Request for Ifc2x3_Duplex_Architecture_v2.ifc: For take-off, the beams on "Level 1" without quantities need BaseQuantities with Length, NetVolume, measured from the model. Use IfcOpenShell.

First a look at what the model holds.

```python
import ifcopenshell
import ifcopenshell.util.element
import ifcopenshell.util.unit

model = ifcopenshell.open("Ifc2x3_Duplex_Architecture_v2.ifc")
print(model.schema)
for unit_type in ("LENGTHUNIT", "AREAUNIT", "VOLUMEUNIT"):
    print(unit_type, ifcopenshell.util.unit.calculate_unit_scale(model, unit_type))
storey = next(s for s in model.by_type("IfcBuildingStorey") if s.Name == "Level 1")
beams = [e for e in ifcopenshell.util.element.get_decomposition(storey) if e.is_a("IfcBeam")]
for e in sorted(beams, key=lambda e: e.id()):
    print(e.id(), e.is_a(), e.Name, list(ifcopenshell.util.element.get_psets(e, qtos_only=True)), sep=" | ")
```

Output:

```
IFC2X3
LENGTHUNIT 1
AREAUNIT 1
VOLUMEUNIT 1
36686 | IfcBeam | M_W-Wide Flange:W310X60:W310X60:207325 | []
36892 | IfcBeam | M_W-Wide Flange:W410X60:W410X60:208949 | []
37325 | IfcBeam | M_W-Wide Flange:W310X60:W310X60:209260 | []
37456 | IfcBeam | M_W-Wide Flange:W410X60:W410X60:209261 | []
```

```python
import ifcopenshell
import ifcopenshell.api.pset
import ifcopenshell.geom
import ifcopenshell.util.element
import ifcopenshell.util.shape
import ifcopenshell.util.unit

model = ifcopenshell.open("Ifc2x3_Duplex_Architecture_v2.ifc")
unit_scale = ifcopenshell.util.unit.calculate_unit_scale(model)
volume_scale = ifcopenshell.util.unit.calculate_unit_scale(model, "VOLUMEUNIT")
settings = ifcopenshell.geom.settings()

storey = next(s for s in model.by_type("IfcBuildingStorey") if s.Name == "Level 1")
beams = [e for e in ifcopenshell.util.element.get_decomposition(storey) if e.is_a("IfcBeam")]

for e in sorted(beams, key=lambda e: e.id()):
    if ifcopenshell.util.element.get_psets(e, qtos_only=True, should_inherit=False):
        continue
    # Geometry comes back in metres, in the element's own axes.
    shape = ifcopenshell.geom.create_shape(settings, e)
    values = {
        "Length": ifcopenshell.util.shape.get_max_xyz(shape.geometry) / unit_scale,
        "NetVolume": ifcopenshell.util.shape.get_volume(shape.geometry) / volume_scale,
    }
    qto = ifcopenshell.api.pset.add_qto(model, product=e, name="BaseQuantities")
    ifcopenshell.api.pset.edit_qto(model, qto=qto, properties=values)
    print(e.id(), {k: round(v, 3) for k, v in values.items()})

model.write("Ifc2x3_Duplex_Architecture_v2_rev.ifc")
```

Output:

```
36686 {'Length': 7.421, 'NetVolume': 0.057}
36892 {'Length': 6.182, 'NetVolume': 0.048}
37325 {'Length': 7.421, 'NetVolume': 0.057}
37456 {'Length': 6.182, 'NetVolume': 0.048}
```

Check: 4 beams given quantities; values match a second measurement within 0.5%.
